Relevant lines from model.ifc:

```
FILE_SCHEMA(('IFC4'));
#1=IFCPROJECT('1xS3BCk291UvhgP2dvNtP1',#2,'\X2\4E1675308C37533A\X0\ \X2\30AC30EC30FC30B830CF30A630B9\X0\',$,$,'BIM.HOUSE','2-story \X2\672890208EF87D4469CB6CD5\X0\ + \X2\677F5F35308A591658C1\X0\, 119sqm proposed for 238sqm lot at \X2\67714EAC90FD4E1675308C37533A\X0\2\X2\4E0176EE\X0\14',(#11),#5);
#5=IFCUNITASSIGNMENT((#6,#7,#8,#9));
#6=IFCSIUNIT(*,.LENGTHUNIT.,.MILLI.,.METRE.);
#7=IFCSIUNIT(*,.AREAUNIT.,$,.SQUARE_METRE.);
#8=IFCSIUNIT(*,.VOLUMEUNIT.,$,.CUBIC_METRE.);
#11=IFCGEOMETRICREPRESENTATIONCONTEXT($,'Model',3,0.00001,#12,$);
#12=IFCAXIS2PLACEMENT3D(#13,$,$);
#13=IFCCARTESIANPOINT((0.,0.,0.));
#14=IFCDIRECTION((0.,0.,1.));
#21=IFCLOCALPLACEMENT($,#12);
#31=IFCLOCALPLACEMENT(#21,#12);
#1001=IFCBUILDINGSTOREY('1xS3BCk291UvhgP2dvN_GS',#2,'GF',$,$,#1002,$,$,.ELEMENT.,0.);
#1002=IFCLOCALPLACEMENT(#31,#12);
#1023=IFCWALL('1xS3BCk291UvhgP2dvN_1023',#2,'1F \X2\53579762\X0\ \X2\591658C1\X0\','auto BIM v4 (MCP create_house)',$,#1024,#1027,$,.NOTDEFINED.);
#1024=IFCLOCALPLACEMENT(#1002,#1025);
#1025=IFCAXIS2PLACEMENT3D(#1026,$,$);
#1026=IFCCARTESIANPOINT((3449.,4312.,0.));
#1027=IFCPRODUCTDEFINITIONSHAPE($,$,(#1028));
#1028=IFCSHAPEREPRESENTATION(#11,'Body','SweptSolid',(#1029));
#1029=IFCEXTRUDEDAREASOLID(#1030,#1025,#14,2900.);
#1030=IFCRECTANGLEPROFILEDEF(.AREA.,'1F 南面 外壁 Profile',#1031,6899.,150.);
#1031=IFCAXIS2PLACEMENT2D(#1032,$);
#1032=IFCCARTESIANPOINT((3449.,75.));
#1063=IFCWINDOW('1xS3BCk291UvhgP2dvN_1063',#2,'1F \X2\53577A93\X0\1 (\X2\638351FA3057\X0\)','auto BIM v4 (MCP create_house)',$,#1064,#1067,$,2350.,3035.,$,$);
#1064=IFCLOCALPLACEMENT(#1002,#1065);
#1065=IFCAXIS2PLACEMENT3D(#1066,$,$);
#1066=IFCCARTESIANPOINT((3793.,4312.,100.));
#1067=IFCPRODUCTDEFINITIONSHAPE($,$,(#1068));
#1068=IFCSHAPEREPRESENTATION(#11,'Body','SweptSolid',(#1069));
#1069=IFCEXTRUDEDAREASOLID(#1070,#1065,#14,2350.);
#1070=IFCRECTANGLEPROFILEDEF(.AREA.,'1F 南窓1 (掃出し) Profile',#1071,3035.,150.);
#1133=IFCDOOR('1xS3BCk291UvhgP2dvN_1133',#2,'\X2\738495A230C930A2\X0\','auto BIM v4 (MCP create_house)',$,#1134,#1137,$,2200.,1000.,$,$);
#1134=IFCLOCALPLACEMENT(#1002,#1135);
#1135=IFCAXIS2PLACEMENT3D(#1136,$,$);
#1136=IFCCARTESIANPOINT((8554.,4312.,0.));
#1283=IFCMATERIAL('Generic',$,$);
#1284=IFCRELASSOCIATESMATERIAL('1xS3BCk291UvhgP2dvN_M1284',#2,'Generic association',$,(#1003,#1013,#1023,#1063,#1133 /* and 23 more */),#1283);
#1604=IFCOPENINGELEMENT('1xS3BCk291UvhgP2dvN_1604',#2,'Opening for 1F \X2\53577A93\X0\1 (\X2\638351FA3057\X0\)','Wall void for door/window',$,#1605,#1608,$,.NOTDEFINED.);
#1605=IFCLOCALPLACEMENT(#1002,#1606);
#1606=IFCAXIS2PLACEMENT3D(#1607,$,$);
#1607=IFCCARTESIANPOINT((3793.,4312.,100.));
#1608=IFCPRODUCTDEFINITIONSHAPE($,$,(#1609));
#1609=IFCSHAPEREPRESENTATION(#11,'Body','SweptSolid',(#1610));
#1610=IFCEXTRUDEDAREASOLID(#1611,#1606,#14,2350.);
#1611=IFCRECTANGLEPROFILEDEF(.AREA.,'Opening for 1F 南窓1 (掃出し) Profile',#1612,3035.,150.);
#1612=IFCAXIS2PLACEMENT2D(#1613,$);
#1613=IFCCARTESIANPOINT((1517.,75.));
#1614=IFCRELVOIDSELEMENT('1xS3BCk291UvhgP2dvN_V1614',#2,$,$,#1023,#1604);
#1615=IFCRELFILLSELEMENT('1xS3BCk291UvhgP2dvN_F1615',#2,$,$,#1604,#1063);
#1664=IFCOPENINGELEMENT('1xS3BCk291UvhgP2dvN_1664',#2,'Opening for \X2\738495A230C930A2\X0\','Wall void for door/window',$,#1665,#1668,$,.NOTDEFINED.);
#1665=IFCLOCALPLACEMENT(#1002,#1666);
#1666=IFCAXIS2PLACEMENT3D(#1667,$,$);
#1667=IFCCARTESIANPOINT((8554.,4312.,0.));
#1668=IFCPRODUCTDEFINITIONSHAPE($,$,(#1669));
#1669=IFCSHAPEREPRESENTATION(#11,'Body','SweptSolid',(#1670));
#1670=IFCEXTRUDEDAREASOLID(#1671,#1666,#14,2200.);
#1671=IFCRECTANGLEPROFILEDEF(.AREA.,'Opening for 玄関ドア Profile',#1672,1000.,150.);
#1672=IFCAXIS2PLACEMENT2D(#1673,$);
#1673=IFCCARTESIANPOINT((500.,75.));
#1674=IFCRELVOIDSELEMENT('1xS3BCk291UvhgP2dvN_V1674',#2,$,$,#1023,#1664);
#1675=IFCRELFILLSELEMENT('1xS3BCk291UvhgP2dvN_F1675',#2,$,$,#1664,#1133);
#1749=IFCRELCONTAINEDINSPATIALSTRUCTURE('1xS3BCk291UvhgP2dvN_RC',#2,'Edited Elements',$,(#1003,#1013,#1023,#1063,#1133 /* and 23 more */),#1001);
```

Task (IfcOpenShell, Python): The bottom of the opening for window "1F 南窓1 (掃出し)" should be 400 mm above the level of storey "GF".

```python
import numpy as np
import ifcopenshell
import ifcopenshell.api.geometry
import ifcopenshell.geom
import ifcopenshell.util.element
import ifcopenshell.util.placement
import ifcopenshell.util.shape
import ifcopenshell.util.unit

model = ifcopenshell.open("model.ifc")
unit_scale = ifcopenshell.util.unit.calculate_unit_scale(model)

window = model.by_id(1063)
opening = window.FillsVoids[0].RelatingOpeningElement
storey = ifcopenshell.util.element.get_container(window, ifc_class="IfcBuildingStorey")
level = ifcopenshell.util.placement.get_local_placement(storey.ObjectPlacement)[2, 3]

# The opening's origin need not be at the sill, so measure its lowest point.
shape = ifcopenshell.geom.create_shape(ifcopenshell.geom.settings(), opening)
bottom = ifcopenshell.util.shape.get_shape_bottom_elevation(shape, shape.geometry) / unit_scale
dz = level + 400.0 - bottom

shift = np.array([0.0, 0.0, dz])
# The window is not placed relative to its opening, so move both.
for product in (opening, window):
    matrix = ifcopenshell.util.placement.get_local_placement(product.ObjectPlacement)
    matrix[:3, 3] += shift
    ifcopenshell.api.geometry.edit_object_placement(model, product=product, matrix=matrix, is_si=False)

print(f"moved by {dz * unit_scale:+.3f} m")

model.write("model_edited.ifc")
```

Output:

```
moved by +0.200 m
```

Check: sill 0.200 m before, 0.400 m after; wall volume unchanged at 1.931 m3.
